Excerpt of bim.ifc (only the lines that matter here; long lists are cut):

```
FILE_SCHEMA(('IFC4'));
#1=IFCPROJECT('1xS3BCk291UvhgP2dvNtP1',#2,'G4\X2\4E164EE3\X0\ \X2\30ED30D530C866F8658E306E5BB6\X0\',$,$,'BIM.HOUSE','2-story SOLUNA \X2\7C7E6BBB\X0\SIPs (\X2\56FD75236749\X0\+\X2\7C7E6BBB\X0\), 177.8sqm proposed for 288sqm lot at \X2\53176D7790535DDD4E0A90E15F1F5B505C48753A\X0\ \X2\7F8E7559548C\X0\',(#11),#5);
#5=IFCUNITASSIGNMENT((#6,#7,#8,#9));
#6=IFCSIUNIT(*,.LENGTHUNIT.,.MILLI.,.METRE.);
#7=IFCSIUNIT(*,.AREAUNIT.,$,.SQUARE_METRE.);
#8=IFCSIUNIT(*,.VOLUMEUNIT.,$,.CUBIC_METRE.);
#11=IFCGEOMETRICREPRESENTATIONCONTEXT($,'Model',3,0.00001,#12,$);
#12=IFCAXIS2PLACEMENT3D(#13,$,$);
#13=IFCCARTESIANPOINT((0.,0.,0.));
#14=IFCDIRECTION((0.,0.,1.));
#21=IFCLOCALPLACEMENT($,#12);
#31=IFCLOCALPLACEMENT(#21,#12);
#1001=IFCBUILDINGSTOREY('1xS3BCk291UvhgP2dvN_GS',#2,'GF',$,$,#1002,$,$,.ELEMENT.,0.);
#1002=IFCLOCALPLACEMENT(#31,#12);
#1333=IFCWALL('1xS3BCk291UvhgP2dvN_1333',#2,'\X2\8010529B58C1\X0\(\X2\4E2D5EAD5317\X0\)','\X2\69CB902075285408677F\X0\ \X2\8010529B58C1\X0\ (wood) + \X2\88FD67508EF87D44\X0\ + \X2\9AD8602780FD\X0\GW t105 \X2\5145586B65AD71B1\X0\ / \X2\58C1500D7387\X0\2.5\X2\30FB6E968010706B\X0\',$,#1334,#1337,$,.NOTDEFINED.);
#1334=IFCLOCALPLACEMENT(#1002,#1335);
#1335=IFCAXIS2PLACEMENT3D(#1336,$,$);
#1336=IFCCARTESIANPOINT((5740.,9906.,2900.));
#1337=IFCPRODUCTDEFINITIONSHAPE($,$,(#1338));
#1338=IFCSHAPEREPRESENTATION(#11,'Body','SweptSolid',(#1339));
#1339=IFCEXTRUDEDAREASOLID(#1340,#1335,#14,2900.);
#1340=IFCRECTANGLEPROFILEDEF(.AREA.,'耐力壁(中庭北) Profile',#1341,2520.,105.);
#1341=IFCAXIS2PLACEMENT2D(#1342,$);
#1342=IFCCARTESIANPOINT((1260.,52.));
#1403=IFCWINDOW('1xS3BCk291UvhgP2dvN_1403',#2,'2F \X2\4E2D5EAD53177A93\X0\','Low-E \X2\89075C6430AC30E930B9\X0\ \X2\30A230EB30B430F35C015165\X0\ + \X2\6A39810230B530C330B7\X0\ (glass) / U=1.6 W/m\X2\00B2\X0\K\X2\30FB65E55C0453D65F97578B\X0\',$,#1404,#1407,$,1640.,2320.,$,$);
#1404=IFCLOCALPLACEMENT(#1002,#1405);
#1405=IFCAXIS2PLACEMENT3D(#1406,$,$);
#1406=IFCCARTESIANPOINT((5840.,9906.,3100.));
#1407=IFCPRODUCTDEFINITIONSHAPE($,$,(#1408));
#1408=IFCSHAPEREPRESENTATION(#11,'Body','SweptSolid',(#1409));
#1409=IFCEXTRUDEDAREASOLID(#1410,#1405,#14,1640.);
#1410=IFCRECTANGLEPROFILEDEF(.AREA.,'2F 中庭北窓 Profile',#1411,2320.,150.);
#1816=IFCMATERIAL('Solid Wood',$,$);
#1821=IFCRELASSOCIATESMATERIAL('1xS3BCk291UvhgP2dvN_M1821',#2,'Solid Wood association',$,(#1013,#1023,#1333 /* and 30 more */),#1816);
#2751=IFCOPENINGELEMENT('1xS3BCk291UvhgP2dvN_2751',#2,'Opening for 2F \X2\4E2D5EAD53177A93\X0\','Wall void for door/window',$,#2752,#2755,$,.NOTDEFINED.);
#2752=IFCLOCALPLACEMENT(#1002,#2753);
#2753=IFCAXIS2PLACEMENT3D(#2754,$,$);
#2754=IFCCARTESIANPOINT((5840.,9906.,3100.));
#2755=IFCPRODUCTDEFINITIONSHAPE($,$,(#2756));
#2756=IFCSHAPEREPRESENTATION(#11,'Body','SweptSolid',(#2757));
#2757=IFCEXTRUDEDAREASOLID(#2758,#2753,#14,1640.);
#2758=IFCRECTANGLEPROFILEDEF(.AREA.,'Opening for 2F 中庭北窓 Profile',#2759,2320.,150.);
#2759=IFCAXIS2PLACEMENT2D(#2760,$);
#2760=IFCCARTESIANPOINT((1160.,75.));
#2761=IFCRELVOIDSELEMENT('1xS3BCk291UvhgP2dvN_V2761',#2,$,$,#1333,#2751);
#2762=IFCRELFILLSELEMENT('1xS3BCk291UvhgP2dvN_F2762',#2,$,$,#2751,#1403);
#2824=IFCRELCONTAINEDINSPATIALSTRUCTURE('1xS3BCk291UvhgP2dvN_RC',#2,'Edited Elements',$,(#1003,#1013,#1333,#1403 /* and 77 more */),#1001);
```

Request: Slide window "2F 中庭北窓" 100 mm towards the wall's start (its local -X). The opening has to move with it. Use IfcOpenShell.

```python
import ifcopenshell
import ifcopenshell.api.geometry
import ifcopenshell.util.placement
import ifcopenshell.util.unit

model = ifcopenshell.open("bim.ifc")
unit_scale = ifcopenshell.util.unit.calculate_unit_scale(model)

window = model.by_guid("1xS3BCk291UvhgP2dvN_1403")
opening = window.FillsVoids[0].RelatingOpeningElement
wall = opening.VoidsElements[0].RelatingBuildingElement

wall_matrix = ifcopenshell.util.placement.get_local_placement(wall.ObjectPlacement)
shift = wall_matrix[:3, 0] * -0.1 / unit_scale
before = ifcopenshell.util.placement.get_local_placement(window.ObjectPlacement)[:3, 3].copy()

# The window is not placed relative to its opening, so move both.
for product in (opening, window):
    matrix = ifcopenshell.util.placement.get_local_placement(product.ObjectPlacement)
    matrix[:3, 3] += shift
    ifcopenshell.api.geometry.edit_object_placement(model, product=product, matrix=matrix, is_si=False)

after = ifcopenshell.util.placement.get_local_placement(window.ObjectPlacement)[:3, 3]
print("window moved by", (after - before).round(3) + 0.0)

model.write("bim_rev.ifc")
```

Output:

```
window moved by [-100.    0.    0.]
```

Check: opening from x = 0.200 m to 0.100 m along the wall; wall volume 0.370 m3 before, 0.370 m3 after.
